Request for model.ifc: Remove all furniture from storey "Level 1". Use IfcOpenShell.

First a look at what the model holds.

```python
import ifcopenshell
import ifcopenshell.util.element

model = ifcopenshell.open("model.ifc")
print(model.schema)
storey = next(s for s in model.by_type("IfcBuildingStorey") if s.Name == "Level 1")
furniture = [e for e in ifcopenshell.util.element.get_decomposition(storey) if e.is_a("IfcFurnishingElement")]
seen = {}
for e in furniture:
    element_type = ifcopenshell.util.element.get_type(e)
    name = element_type.Name if element_type not in (None, e) else None
    seen[name] = seen.get(name, 0) + 1
for name, count in sorted(seen.items(), key=str):
    print(count, "x", name)
```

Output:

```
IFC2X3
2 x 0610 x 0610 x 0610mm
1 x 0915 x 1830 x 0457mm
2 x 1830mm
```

```python
import ifcopenshell
import ifcopenshell.api.root
import ifcopenshell.util.element

model = ifcopenshell.open("model.ifc")

storey = next(s for s in model.by_type("IfcBuildingStorey") if s.Name == "Level 1")
furniture = [e for e in ifcopenshell.util.element.get_decomposition(storey) if e.is_a("IfcFurnishingElement")]

for e in furniture:
    ifcopenshell.api.root.remove_product(model, product=e)
print(len(furniture), "removed")

model.write("model-out.ifc")
```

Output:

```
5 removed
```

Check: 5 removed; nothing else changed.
